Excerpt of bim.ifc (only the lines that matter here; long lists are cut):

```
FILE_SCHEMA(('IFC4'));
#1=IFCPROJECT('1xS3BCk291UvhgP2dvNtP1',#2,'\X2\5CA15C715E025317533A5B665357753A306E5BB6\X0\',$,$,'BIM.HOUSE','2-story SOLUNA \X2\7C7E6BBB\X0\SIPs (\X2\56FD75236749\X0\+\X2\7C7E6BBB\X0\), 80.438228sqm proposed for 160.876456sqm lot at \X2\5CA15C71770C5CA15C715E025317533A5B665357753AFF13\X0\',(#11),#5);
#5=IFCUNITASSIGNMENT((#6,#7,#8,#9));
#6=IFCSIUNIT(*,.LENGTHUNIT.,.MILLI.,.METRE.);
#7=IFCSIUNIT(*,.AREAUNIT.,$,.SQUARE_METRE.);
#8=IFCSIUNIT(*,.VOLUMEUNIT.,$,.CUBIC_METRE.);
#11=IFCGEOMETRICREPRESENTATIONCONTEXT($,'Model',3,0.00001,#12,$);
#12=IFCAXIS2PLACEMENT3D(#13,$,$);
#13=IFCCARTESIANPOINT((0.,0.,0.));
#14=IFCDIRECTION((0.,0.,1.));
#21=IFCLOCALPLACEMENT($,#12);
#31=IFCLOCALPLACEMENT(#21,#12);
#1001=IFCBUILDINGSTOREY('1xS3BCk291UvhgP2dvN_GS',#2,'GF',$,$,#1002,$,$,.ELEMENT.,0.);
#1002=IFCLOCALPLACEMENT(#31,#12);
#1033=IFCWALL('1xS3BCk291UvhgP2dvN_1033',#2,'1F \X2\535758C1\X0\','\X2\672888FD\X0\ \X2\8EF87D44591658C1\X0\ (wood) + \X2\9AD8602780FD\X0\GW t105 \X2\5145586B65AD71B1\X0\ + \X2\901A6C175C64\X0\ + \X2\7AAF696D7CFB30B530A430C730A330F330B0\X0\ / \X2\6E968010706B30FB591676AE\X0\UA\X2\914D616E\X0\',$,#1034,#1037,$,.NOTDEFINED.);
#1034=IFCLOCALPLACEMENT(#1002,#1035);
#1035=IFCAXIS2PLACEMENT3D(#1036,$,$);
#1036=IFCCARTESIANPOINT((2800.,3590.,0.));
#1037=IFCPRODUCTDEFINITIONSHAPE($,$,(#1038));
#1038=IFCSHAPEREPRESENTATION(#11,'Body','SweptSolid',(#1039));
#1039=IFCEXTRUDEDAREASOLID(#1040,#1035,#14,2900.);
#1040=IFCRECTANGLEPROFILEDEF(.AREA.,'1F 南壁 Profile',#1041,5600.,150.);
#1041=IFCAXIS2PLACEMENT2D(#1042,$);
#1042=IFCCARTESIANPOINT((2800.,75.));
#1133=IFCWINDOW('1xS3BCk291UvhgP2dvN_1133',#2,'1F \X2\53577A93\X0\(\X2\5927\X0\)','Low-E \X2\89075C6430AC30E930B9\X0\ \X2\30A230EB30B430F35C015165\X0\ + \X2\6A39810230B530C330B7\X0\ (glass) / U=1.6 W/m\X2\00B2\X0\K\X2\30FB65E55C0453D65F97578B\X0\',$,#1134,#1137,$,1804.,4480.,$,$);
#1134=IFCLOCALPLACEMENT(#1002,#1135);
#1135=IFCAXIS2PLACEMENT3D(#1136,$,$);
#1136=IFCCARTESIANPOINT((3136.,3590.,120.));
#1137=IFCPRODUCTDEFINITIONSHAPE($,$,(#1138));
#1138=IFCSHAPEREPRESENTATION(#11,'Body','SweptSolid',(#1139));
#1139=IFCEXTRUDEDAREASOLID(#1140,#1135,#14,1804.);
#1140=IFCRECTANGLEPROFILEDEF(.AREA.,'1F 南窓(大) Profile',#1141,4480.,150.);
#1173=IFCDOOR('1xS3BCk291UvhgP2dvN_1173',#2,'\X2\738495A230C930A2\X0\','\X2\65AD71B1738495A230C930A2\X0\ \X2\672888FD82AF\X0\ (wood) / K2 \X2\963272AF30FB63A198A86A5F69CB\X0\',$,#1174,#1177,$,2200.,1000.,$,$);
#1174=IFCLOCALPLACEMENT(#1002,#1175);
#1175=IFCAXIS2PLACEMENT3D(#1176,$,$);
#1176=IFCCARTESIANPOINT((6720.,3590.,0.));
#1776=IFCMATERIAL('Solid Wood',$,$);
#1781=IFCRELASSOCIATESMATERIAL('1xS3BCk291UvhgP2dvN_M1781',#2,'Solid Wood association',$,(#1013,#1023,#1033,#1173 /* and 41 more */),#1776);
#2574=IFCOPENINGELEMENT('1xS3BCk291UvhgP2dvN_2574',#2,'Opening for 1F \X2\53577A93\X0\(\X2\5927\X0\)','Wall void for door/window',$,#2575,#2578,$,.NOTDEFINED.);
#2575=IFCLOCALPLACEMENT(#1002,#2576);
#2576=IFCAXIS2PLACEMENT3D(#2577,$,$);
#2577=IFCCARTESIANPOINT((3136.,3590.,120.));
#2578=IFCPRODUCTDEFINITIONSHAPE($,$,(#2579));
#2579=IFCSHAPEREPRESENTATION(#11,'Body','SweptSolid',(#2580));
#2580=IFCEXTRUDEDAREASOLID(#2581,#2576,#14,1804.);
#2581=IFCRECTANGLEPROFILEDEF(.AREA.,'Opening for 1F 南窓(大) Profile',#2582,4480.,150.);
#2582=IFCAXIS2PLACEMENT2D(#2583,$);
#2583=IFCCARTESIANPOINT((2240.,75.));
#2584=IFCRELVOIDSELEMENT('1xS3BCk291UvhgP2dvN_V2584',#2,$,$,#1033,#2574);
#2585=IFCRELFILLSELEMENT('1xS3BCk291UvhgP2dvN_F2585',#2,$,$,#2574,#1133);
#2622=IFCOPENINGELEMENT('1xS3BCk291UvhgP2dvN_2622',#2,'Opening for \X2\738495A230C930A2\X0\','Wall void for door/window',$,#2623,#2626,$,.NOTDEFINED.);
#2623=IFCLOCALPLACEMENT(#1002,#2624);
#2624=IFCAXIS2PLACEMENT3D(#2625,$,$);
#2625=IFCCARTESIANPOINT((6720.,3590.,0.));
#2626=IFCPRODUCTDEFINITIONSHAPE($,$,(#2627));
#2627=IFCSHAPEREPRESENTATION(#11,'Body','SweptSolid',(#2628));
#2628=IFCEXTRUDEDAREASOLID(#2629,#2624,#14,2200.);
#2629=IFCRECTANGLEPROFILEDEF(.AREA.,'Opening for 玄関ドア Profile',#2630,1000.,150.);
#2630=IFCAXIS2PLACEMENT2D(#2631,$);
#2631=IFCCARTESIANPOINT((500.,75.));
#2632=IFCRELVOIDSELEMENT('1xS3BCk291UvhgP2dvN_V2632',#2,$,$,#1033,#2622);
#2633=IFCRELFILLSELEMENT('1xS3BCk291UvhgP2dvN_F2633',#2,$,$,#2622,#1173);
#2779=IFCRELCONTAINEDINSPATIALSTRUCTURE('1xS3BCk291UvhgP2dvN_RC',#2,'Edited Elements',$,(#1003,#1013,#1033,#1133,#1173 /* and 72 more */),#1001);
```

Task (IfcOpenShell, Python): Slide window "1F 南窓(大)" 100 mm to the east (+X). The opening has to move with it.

```python
import ifcopenshell
import ifcopenshell.api.geometry
import ifcopenshell.util.placement

model = ifcopenshell.open("bim.ifc")

window = model.by_guid("1xS3BCk291UvhgP2dvN_1133")
opening = window.FillsVoids[0].RelatingOpeningElement
wall = opening.VoidsElements[0].RelatingBuildingElement

wall_matrix = ifcopenshell.util.placement.get_local_placement(wall.ObjectPlacement)
shift = wall_matrix[:3, 0] * 100.0
before = ifcopenshell.util.placement.get_local_placement(window.ObjectPlacement)[:3, 3].copy()

# The window is not placed relative to its opening, so move both.
for product in (opening, window):
    matrix = ifcopenshell.util.placement.get_local_placement(product.ObjectPlacement)
    matrix[:3, 3] += shift
    ifcopenshell.api.geometry.edit_object_placement(model, product=product, matrix=matrix, is_si=False)

after = ifcopenshell.util.placement.get_local_placement(window.ObjectPlacement)[:3, 3]
print("window moved by", (after - before).round(3) + 0.0)

model.write("bim_edited.ifc")
```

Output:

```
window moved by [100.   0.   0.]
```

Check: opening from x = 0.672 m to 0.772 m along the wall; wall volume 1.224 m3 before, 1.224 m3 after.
